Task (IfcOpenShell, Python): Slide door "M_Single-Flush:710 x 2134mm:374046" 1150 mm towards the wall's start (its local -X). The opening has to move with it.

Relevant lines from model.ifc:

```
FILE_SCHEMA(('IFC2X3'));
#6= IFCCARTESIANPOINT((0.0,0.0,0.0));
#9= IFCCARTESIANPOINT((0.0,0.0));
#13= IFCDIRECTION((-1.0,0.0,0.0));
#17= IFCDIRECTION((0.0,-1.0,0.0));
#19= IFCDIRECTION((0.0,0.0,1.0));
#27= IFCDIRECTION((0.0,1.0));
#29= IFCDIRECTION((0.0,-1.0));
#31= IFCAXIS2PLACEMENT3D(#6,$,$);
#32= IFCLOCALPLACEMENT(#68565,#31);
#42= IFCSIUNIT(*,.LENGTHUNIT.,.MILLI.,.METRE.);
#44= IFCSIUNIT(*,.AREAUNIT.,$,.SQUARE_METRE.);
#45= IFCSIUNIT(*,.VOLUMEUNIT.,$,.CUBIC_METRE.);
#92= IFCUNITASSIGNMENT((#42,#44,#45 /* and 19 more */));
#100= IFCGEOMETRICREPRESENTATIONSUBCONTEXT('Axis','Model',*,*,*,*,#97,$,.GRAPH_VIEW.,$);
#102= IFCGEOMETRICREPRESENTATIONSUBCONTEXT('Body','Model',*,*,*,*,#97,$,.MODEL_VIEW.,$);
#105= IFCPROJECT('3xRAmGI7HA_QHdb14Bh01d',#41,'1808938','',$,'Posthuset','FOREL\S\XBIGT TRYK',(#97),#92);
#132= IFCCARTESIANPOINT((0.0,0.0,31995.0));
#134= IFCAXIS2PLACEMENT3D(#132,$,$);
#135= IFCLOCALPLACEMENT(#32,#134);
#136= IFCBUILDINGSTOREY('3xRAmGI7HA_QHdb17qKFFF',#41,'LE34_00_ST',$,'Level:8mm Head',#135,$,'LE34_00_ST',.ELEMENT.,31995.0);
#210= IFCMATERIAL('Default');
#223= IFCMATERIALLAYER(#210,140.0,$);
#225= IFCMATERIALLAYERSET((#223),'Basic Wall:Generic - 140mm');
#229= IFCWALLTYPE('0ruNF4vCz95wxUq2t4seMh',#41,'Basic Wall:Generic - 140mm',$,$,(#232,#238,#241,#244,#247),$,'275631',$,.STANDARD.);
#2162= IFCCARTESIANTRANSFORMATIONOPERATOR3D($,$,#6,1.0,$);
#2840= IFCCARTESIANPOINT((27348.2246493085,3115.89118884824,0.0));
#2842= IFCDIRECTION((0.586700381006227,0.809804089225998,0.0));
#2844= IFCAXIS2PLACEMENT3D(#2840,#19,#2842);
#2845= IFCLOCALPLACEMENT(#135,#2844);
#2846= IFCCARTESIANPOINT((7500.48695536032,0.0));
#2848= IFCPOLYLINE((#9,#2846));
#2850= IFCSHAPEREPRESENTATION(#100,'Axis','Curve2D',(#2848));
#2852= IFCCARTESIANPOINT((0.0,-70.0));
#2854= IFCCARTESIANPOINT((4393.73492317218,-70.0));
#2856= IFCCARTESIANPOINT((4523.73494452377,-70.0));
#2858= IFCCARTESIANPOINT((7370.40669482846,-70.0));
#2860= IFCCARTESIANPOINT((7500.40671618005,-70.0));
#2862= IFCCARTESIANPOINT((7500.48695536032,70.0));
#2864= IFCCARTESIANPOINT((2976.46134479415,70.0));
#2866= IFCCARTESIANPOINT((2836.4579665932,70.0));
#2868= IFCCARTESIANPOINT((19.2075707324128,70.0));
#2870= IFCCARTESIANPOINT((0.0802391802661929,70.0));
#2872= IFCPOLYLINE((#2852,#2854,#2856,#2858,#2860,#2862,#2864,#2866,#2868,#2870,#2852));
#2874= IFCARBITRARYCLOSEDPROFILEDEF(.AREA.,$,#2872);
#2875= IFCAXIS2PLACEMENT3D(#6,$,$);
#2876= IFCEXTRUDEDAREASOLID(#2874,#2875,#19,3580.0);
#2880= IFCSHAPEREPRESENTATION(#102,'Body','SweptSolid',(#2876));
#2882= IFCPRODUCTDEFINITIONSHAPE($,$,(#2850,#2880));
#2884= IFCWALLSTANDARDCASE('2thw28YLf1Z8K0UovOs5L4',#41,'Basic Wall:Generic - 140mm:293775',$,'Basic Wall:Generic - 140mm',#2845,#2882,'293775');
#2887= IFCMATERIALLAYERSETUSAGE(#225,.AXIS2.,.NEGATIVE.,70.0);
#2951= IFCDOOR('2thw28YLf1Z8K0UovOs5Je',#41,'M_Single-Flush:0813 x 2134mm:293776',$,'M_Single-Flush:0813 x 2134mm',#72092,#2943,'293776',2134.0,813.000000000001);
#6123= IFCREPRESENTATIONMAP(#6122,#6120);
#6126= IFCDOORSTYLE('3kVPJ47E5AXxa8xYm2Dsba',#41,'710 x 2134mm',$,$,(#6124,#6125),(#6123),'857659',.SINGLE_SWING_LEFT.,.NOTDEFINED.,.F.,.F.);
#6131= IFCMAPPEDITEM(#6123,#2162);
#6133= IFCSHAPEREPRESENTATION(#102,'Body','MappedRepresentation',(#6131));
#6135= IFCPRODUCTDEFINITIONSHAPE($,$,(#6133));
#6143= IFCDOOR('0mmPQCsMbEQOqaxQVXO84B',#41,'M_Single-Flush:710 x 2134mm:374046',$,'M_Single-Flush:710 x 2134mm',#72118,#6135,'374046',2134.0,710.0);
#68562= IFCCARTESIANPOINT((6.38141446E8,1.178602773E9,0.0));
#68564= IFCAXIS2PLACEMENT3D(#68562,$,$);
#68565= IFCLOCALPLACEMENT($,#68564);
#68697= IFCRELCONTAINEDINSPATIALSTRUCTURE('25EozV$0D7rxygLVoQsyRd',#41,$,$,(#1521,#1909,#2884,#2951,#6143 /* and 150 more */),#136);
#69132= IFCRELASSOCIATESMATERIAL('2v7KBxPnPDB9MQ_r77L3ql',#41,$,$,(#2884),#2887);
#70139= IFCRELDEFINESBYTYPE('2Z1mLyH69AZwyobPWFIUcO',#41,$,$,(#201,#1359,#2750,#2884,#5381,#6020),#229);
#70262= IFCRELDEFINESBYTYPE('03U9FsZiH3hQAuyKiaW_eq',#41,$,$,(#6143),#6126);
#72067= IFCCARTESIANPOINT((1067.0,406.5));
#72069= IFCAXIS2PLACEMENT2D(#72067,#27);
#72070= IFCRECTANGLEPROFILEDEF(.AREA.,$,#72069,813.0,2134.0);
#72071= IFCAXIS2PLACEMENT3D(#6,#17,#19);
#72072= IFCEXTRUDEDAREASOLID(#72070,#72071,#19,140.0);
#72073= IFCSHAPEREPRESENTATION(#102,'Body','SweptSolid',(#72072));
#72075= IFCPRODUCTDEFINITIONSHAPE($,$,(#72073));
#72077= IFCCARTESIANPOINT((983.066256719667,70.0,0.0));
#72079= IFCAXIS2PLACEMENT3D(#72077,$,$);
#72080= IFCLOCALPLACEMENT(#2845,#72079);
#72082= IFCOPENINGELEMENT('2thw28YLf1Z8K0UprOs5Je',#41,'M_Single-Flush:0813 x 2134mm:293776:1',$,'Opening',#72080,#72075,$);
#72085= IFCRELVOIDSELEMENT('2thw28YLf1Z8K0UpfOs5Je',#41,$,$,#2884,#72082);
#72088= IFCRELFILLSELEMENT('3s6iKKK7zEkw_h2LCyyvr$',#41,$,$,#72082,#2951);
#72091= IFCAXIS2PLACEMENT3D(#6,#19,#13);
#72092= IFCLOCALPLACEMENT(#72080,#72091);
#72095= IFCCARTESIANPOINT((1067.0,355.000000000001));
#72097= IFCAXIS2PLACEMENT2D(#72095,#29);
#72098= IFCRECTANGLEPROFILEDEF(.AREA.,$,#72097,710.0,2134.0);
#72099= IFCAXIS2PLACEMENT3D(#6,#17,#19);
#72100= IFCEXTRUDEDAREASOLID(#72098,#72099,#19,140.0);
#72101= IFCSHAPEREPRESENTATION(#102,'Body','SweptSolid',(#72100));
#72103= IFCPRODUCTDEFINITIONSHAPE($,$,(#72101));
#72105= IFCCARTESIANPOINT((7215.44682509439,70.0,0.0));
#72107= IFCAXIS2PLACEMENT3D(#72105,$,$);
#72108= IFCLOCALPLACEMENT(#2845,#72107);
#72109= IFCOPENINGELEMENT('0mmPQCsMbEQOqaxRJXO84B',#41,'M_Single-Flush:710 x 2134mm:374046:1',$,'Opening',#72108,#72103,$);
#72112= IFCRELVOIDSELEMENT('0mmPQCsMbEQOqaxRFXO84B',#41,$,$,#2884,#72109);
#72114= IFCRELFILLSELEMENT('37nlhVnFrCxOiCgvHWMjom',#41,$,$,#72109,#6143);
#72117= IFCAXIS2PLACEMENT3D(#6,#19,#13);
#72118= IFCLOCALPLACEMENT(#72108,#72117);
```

```python
import ifcopenshell
import ifcopenshell.api.geometry
import ifcopenshell.util.placement
import ifcopenshell.util.unit

model = ifcopenshell.open("model.ifc")
unit_scale = ifcopenshell.util.unit.calculate_unit_scale(model)

door = model.by_guid("0mmPQCsMbEQOqaxQVXO84B")
opening = door.FillsVoids[0].RelatingOpeningElement
wall = opening.VoidsElements[0].RelatingBuildingElement

wall_matrix = ifcopenshell.util.placement.get_local_placement(wall.ObjectPlacement)
shift = wall_matrix[:3, 0] * -1.15 / unit_scale
before = ifcopenshell.util.placement.get_local_placement(door.ObjectPlacement)[:3, 3].copy()

# The door is placed relative to its opening, so it follows when the opening moves.
matrix = ifcopenshell.util.placement.get_local_placement(opening.ObjectPlacement)
matrix[:3, 3] += shift
ifcopenshell.api.geometry.edit_object_placement(
    model, product=opening, matrix=matrix, is_si=False, should_transform_children=True
)

after = ifcopenshell.util.placement.get_local_placement(door.ObjectPlacement)[:3, 3]
print("door moved by", (after - before).round(3) + 0.0)

model.write("model_rev.ifc")
```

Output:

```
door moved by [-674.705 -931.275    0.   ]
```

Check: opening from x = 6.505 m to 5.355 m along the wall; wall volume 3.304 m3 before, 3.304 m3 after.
